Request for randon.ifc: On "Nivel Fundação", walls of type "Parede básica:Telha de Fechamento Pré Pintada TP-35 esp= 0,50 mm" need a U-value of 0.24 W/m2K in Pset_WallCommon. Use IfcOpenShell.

First a look at what the model holds.

```python
import ifcopenshell
import ifcopenshell.util.element

model = ifcopenshell.open("randon.ifc")
print(model.schema)
storey = next(s for s in model.by_type("IfcBuildingStorey") if s.Name == "Nivel Fundação")
walls = [e for e in ifcopenshell.util.element.get_decomposition(storey) if e.is_a("IfcWall")]
seen = {}
for e in walls:
    element_type = ifcopenshell.util.element.get_type(e)
    key = (element_type.Name if element_type != e and element_type else None, ifcopenshell.util.element.get_pset(e, "Pset_WallCommon", "ThermalTransmittance"))
    seen[key] = seen.get(key, 0) + 1
for (name, value), count in sorted(seen.items(), key=str):
    print(count, "x", name, "|", value)
```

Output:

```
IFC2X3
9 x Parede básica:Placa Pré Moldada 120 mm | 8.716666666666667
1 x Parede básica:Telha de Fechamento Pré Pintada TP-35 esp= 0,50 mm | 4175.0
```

```python
import ifcopenshell
import ifcopenshell.api.pset
import ifcopenshell.util.element

model = ifcopenshell.open("randon.ifc")

storey = next(s for s in model.by_type("IfcBuildingStorey") if s.Name == "Nivel Fundação")
walls = [e for e in ifcopenshell.util.element.get_decomposition(storey) if e.is_a("IfcWall")]

count = 0
for e in walls:
    element_type = ifcopenshell.util.element.get_type(e)
    if element_type in (None, e) or element_type.Name != "Parede básica:Telha de Fechamento Pré Pintada TP-35 esp= 0,50 mm":
        continue
    # add_pset returns the element's existing set when there is one.
    pset = ifcopenshell.api.pset.add_pset(model, product=e, name="Pset_WallCommon")
    ifcopenshell.api.pset.edit_pset(model, pset=pset, properties={"ThermalTransmittance": 0.24})
    count += 1

print(count, "walls updated")

model.write("randon_updated.ifc")
```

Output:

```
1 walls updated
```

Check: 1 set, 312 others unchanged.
